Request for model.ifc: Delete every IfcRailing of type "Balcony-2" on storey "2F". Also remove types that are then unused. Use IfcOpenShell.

First a look at what the model holds.

```python
import ifcopenshell
import ifcopenshell.util.element

model = ifcopenshell.open("model.ifc")
print(model.schema)
storey = next(s for s in model.by_type("IfcBuildingStorey") if s.Name == "2F")
railings = [e for e in ifcopenshell.util.element.get_decomposition(storey) if e.is_a("IfcRailing")]
seen = {}
for e in railings:
    element_type = ifcopenshell.util.element.get_type(e)
    name = element_type.Name if element_type not in (None, e) else None
    seen[name] = seen.get(name, 0) + 1
for name, count in sorted(seen.items(), key=str):
    print(count, "x", name)
```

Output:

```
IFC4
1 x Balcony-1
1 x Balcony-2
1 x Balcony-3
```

```python
import ifcopenshell
import ifcopenshell.api.root
import ifcopenshell.util.element

model = ifcopenshell.open("model.ifc")

storey = next(s for s in model.by_type("IfcBuildingStorey") if s.Name == "2F")
railings = [e for e in ifcopenshell.util.element.get_decomposition(storey) if e.is_a("IfcRailing")]
targets = [e for e in railings if (t := ifcopenshell.util.element.get_type(e)) not in (None, e) and t.Name == "Balcony-2"]
types = {ifcopenshell.util.element.get_type(e) for e in targets} - {None, *targets}

for e in targets:
    ifcopenshell.api.root.remove_product(model, product=e)
print(len(targets), "removed")

unused = [t for t in types if not ifcopenshell.util.element.get_types(t)]
for t in unused:
    ifcopenshell.api.root.remove_product(model, product=t)
print(len(unused), "unused types removed")

model.write("model_rev.ifc")
```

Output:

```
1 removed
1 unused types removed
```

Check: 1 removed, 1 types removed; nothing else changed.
